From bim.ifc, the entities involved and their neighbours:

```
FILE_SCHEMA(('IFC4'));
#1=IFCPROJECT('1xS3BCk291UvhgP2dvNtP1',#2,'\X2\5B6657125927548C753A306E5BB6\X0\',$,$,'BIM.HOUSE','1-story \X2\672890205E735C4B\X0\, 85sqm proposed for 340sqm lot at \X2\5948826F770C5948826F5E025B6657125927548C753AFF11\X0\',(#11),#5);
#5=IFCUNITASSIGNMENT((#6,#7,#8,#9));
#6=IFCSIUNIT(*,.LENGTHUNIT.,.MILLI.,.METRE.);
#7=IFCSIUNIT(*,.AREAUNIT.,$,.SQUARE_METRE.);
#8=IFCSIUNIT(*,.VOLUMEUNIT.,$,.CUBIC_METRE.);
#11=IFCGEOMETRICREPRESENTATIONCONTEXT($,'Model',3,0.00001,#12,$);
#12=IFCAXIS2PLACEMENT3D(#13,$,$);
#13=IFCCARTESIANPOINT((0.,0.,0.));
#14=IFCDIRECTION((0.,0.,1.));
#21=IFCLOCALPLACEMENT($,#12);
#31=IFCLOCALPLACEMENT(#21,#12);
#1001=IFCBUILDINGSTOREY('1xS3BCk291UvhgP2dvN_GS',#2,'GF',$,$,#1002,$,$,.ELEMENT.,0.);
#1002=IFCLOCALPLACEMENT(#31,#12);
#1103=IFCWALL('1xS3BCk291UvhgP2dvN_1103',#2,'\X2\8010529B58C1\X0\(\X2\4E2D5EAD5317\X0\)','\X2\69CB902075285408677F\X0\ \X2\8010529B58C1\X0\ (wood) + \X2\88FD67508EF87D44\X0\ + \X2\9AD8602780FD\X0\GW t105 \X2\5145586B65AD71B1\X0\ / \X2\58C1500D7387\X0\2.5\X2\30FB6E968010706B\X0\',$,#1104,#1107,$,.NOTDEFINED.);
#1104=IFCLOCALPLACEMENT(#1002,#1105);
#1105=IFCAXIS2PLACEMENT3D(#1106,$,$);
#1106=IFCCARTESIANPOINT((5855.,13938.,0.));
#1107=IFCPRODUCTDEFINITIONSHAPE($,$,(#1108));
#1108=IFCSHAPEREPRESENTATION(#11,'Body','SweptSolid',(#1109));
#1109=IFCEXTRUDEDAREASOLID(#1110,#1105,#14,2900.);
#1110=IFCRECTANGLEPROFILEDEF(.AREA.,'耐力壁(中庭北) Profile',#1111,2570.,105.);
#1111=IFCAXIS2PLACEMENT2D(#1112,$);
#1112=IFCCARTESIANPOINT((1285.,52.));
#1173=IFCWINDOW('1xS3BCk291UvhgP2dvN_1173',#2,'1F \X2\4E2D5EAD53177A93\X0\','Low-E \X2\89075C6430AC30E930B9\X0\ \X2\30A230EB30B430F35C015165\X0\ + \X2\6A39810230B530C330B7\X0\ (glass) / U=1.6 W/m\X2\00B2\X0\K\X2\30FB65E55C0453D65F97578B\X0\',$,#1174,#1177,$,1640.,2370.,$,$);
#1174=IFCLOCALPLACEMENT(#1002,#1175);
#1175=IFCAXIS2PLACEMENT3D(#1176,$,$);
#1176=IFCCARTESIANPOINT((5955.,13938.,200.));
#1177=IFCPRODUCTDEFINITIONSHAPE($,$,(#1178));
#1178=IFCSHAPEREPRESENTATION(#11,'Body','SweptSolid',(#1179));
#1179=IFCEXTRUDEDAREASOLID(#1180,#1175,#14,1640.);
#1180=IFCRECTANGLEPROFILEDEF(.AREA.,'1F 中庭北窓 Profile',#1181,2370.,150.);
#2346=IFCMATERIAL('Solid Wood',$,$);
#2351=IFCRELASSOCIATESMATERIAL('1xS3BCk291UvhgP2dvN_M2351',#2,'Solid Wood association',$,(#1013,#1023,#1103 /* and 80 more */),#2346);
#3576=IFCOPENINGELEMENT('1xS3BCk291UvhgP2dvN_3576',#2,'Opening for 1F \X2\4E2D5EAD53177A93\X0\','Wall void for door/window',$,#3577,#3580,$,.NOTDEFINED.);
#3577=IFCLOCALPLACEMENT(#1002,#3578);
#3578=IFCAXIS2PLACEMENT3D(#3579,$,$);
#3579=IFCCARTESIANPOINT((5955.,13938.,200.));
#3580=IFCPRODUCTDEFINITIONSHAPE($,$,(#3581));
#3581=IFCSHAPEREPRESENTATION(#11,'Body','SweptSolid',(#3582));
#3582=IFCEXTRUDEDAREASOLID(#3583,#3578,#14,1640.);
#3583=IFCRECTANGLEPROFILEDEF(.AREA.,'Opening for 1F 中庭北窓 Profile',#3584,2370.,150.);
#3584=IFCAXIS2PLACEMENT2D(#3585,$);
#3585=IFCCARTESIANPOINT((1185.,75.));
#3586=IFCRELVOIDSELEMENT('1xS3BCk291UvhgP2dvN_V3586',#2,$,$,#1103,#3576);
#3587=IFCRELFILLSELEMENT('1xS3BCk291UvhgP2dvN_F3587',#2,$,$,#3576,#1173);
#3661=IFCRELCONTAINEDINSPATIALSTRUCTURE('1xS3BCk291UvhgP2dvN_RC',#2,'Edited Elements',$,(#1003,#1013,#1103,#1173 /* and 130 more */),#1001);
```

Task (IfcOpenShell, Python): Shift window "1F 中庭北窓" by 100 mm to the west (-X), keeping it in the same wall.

```python
import ifcopenshell
import ifcopenshell.api.geometry
import ifcopenshell.util.placement
import ifcopenshell.util.unit

model = ifcopenshell.open("bim.ifc")
unit_scale = ifcopenshell.util.unit.calculate_unit_scale(model)

window = model.by_guid("1xS3BCk291UvhgP2dvN_1173")
opening = window.FillsVoids[0].RelatingOpeningElement
wall = opening.VoidsElements[0].RelatingBuildingElement

wall_matrix = ifcopenshell.util.placement.get_local_placement(wall.ObjectPlacement)
shift = wall_matrix[:3, 0] * -0.1 / unit_scale
before = ifcopenshell.util.placement.get_local_placement(window.ObjectPlacement)[:3, 3].copy()

# The window is not placed relative to its opening, so move both.
for product in (opening, window):
    matrix = ifcopenshell.util.placement.get_local_placement(product.ObjectPlacement)
    matrix[:3, 3] += shift
    ifcopenshell.api.geometry.edit_object_placement(model, product=product, matrix=matrix, is_si=False)

after = ifcopenshell.util.placement.get_local_placement(window.ObjectPlacement)[:3, 3]
print("window moved by", (after - before).round(3) + 0.0)

model.write("bim_rev.ifc")
```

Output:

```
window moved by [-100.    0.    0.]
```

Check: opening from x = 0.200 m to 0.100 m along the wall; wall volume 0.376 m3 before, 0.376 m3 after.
